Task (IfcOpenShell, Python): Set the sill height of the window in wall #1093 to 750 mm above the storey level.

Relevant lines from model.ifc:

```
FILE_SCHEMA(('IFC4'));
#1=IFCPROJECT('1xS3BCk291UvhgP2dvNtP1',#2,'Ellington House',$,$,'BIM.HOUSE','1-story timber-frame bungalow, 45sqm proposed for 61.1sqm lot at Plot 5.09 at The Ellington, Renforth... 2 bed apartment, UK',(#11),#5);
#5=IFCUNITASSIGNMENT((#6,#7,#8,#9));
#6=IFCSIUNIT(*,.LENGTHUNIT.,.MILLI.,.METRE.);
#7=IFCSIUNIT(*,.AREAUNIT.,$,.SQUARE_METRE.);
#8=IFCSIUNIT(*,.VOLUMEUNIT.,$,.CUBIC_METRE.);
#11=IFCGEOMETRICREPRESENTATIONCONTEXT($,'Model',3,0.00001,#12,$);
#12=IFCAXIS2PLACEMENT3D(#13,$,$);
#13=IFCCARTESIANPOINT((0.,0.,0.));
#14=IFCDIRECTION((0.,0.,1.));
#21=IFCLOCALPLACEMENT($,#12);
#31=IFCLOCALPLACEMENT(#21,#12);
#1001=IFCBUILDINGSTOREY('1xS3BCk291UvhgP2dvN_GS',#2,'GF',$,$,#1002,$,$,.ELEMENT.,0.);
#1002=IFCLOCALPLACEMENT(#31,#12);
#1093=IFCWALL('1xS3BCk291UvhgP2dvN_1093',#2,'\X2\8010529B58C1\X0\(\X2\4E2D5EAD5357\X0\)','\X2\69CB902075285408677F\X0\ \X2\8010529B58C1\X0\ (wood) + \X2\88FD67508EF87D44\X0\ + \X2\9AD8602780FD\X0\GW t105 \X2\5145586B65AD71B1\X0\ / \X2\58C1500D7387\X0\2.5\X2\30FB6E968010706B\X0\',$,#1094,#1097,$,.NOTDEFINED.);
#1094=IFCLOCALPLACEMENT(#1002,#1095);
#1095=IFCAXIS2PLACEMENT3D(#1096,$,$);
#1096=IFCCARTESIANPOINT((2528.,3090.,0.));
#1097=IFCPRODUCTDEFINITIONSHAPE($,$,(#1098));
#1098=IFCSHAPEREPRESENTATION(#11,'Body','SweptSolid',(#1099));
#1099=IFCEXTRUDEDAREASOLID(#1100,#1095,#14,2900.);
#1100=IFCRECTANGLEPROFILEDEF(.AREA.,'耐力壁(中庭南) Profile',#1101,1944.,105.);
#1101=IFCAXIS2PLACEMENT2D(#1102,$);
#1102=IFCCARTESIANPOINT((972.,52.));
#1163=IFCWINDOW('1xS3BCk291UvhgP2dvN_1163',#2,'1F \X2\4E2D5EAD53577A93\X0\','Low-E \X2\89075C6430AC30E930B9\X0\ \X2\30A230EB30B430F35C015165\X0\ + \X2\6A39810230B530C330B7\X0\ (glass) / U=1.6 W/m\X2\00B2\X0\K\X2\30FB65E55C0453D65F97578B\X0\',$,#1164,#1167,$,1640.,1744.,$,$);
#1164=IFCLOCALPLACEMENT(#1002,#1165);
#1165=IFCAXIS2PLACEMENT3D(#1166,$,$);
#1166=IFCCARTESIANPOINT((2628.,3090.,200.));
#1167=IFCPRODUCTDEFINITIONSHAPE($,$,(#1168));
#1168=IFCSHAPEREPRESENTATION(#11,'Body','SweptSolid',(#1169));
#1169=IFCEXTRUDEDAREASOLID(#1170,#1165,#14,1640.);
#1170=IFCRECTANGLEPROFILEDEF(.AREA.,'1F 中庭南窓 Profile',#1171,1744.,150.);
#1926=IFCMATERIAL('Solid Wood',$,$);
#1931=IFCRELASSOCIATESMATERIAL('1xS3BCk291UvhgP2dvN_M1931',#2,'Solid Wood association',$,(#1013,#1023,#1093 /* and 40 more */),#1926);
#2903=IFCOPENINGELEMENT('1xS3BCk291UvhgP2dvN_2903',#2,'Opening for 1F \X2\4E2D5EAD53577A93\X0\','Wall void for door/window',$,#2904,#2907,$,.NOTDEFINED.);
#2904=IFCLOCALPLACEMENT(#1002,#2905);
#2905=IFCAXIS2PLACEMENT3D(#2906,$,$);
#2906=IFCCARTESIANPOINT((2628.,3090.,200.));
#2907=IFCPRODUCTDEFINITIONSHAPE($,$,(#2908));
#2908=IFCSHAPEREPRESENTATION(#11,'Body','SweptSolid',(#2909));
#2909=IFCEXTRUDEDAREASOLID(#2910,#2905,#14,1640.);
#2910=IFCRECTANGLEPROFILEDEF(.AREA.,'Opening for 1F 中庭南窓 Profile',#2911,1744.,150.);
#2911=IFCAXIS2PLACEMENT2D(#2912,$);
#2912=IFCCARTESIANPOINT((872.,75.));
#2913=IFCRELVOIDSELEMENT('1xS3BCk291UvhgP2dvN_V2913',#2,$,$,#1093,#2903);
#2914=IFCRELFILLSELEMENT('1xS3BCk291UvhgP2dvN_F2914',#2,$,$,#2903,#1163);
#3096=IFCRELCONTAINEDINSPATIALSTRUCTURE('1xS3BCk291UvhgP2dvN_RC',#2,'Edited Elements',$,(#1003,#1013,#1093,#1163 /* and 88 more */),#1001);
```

```python
import numpy as np
import ifcopenshell
import ifcopenshell.api.geometry
import ifcopenshell.geom
import ifcopenshell.util.element
import ifcopenshell.util.placement
import ifcopenshell.util.shape
import ifcopenshell.util.unit

model = ifcopenshell.open("model.ifc")
unit_scale = ifcopenshell.util.unit.calculate_unit_scale(model)

window = model.by_guid("1xS3BCk291UvhgP2dvN_1163")
opening = window.FillsVoids[0].RelatingOpeningElement
storey = ifcopenshell.util.element.get_container(window, ifc_class="IfcBuildingStorey")
level = ifcopenshell.util.placement.get_local_placement(storey.ObjectPlacement)[2, 3]

# The opening's origin need not be at the sill, so measure its lowest point.
shape = ifcopenshell.geom.create_shape(ifcopenshell.geom.settings(), opening)
bottom = ifcopenshell.util.shape.get_shape_bottom_elevation(shape, shape.geometry) / unit_scale
dz = level + 0.75 / unit_scale - bottom

shift = np.array([0.0, 0.0, dz])
# The window is not placed relative to its opening, so move both.
for product in (opening, window):
    matrix = ifcopenshell.util.placement.get_local_placement(product.ObjectPlacement)
    matrix[:3, 3] += shift
    ifcopenshell.api.geometry.edit_object_placement(model, product=product, matrix=matrix, is_si=False)

print(f"moved by {dz * unit_scale:+.3f} m")

model.write("model_v2.ifc")
```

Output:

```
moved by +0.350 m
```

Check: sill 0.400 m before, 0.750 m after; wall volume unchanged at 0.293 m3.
